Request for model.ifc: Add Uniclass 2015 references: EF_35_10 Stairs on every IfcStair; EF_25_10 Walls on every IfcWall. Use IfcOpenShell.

First a look at what the model holds.

```python
import ifcopenshell

model = ifcopenshell.open("model.ifc")
print(model.schema)
print("classifications:", [c.Name for c in model.by_type("IfcClassification")])
for ifc_class in ("IfcDoor", "IfcRoof", "IfcStair", "IfcWall", "IfcWindow"):
    print(ifc_class, len(model.by_type(ifc_class)))
```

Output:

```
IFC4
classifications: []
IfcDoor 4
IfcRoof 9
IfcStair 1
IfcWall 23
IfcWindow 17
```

```python
import ifcopenshell
import ifcopenshell.api.classification

model = ifcopenshell.open("model.ifc")

system = ifcopenshell.api.classification.add_classification(model, classification="Uniclass 2015")

codes = {
    "IfcStair": ("EF_35_10", "Stairs"),
    "IfcWall": ("EF_25_10", "Walls"),
}
for ifc_class, (code, name) in codes.items():
    products = model.by_type(ifc_class)
    ifcopenshell.api.classification.add_reference(
        model, products=products, classification=system, identification=code, name=name
    )
    print(code, len(products))

model.write("model_edited.ifc")
```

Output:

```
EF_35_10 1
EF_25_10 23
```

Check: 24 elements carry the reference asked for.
